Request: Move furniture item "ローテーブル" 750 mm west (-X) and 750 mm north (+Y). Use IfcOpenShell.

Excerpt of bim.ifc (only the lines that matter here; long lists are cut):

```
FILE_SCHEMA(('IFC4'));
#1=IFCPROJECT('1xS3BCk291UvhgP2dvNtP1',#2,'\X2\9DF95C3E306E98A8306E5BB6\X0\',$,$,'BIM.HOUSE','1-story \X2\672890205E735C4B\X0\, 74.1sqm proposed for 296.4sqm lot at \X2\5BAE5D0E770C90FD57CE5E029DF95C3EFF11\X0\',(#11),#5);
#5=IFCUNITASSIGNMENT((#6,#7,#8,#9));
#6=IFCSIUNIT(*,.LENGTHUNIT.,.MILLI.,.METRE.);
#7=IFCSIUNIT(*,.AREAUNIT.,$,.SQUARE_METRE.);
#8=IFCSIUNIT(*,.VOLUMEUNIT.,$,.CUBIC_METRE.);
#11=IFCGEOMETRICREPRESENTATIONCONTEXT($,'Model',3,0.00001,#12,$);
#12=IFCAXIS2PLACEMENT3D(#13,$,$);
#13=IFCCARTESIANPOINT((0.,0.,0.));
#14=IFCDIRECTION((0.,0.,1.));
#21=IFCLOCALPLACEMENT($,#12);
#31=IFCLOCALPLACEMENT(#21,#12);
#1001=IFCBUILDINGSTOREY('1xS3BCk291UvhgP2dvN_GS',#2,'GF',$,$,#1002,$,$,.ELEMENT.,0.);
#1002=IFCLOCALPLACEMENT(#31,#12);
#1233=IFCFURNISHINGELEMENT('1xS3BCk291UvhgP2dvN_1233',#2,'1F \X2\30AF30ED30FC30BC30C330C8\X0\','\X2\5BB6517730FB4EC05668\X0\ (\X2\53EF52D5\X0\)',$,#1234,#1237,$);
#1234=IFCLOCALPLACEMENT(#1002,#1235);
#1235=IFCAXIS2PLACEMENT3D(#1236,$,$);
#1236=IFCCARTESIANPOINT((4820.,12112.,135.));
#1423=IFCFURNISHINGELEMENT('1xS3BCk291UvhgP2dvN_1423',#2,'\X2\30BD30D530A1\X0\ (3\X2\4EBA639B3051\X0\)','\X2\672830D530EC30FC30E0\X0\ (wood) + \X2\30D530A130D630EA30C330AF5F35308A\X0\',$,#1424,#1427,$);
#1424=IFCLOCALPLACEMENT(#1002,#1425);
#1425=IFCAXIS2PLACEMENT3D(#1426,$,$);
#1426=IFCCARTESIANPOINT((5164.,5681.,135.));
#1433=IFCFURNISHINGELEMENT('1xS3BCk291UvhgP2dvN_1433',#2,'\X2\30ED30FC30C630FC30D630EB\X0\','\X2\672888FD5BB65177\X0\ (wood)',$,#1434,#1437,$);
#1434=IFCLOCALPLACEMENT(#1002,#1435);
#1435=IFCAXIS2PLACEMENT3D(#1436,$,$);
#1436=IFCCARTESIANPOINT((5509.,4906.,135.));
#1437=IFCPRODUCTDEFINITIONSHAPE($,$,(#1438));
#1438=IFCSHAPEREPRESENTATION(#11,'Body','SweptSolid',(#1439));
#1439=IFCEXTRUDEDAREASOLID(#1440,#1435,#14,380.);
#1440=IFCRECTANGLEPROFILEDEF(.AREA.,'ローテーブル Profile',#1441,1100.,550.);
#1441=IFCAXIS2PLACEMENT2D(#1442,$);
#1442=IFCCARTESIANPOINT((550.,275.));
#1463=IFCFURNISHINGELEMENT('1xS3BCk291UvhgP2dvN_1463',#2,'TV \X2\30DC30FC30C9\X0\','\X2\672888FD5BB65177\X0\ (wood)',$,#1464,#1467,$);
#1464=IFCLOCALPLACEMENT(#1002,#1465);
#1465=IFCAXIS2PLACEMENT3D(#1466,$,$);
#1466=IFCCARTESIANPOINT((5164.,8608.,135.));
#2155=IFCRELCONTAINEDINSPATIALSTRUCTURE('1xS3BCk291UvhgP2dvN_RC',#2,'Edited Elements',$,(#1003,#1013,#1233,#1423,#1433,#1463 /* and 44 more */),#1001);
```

```python
import ifcopenshell
import ifcopenshell.api.geometry
import ifcopenshell.util.placement

model = ifcopenshell.open("bim.ifc")

item = model.by_guid("1xS3BCk291UvhgP2dvN_1433")
matrix = ifcopenshell.util.placement.get_local_placement(item.ObjectPlacement)
matrix[0, 3] -= 750.0
matrix[1, 3] += 750.0
ifcopenshell.api.geometry.edit_object_placement(model, product=item, matrix=matrix, is_si=False)

print(ifcopenshell.util.placement.get_local_placement(item.ObjectPlacement).round(3) + 0.0)

model.write("bim_rev.ifc")
```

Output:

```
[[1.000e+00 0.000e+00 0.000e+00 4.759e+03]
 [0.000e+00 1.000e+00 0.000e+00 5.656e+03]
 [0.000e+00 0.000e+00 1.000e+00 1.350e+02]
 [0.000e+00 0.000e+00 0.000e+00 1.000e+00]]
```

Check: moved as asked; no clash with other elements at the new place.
